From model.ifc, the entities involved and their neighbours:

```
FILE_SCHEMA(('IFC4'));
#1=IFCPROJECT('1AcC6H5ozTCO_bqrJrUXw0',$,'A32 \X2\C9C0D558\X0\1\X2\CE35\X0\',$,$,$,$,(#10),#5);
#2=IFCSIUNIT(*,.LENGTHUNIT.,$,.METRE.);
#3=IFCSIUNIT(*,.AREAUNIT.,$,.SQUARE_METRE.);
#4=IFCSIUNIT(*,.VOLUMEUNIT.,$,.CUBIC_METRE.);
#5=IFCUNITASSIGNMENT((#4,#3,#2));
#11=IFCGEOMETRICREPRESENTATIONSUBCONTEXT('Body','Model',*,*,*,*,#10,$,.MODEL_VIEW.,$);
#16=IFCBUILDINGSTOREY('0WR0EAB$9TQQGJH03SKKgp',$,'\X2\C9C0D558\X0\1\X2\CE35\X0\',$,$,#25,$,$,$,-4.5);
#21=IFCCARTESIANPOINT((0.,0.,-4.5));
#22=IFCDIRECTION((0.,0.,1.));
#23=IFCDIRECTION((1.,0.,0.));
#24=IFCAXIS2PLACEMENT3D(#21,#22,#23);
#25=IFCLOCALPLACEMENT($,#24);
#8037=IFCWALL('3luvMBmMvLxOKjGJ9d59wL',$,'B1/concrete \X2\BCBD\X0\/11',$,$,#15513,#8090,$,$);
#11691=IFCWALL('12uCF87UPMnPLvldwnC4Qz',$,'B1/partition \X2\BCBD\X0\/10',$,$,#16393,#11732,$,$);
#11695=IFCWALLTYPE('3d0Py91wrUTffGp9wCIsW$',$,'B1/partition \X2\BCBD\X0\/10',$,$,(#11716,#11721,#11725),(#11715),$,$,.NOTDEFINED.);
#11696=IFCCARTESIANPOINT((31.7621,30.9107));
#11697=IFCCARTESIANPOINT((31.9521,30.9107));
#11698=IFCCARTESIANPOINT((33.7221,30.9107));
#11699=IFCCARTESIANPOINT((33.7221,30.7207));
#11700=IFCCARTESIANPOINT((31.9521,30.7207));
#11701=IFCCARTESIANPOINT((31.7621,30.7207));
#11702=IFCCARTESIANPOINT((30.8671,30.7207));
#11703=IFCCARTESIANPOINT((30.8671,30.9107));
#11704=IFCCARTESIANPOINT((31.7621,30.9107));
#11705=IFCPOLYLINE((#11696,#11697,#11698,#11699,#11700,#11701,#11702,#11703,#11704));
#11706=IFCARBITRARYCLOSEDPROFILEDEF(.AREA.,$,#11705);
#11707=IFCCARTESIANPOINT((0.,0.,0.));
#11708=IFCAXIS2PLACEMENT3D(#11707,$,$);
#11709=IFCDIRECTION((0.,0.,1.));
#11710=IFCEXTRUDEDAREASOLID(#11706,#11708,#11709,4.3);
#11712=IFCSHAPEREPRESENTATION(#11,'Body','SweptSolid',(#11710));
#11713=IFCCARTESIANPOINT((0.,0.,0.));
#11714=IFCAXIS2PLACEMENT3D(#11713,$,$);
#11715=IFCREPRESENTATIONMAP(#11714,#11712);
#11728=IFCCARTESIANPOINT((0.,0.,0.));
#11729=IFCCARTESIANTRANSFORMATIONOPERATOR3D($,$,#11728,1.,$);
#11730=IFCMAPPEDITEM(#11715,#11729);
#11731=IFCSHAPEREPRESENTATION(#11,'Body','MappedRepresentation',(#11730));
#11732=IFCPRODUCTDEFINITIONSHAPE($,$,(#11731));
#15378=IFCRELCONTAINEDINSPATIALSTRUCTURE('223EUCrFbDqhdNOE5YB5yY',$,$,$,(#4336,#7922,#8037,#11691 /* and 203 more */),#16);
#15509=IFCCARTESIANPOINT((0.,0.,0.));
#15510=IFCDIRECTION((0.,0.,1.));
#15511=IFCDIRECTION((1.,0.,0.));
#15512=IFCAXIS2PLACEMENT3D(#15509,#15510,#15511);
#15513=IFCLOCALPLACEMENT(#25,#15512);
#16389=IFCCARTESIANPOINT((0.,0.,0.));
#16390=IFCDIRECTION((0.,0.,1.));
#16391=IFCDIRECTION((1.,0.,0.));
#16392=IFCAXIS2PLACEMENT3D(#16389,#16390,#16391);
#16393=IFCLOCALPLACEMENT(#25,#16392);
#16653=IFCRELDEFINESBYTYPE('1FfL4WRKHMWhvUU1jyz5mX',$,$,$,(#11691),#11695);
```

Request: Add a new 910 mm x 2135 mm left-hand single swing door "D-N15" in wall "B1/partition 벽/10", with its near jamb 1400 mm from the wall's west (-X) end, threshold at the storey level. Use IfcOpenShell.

```python
import numpy as np
import ifcopenshell
import ifcopenshell.api.feature
import ifcopenshell.api.geometry
import ifcopenshell.api.root
import ifcopenshell.api.spatial
import ifcopenshell.geom
import ifcopenshell.util.element
import ifcopenshell.util.placement
import ifcopenshell.util.representation
import ifcopenshell.util.shape
import ifcopenshell.util.unit

model = ifcopenshell.open("model.ifc")
unit_scale = ifcopenshell.util.unit.calculate_unit_scale(model)
settings = ifcopenshell.geom.settings()


def volume(element):
    """Net volume in cubic metres, openings subtracted."""
    shape = ifcopenshell.geom.create_shape(settings, element)
    return ifcopenshell.util.shape.get_volume(shape.geometry)


wall = model.by_guid("12uCF87UPMnPLvldwnC4Qz")
storey = ifcopenshell.util.element.get_container(wall, ifc_class="IfcBuildingStorey")
context = ifcopenshell.util.representation.get_context(model, "Model", "Body", "MODEL_VIEW")
before = volume(wall)

width, height, from_end, sill = 0.91, 2.135, 1.4, 0.0  # metres

# The wall runs along its own X axis, and the end named is its -X end.
wall_shape = ifcopenshell.geom.create_shape(settings, wall)
x, y, z = ifcopenshell.util.shape.get_vertices(wall_shape.geometry).T
start = x.min() + from_end
face, thickness = float(y.min()), float(y.max() - y.min())
wall_matrix = ifcopenshell.util.placement.get_local_placement(wall.ObjectPlacement)
level = ifcopenshell.util.placement.get_local_placement(storey.ObjectPlacement)[2, 3]


def in_wall(x, y):
    """Placement at x, y metres in the wall's axes, at sill height."""
    matrix = wall_matrix.copy()
    matrix[:, 3] = wall_matrix @ np.array([x / unit_scale, y / unit_scale, 0.0, 1.0])
    matrix[2, 3] = level + sill / unit_scale
    return matrix


# Opening: a box that overshoots both wall faces by 50 mm.
opening = ifcopenshell.api.root.create_entity(model, ifc_class="IfcOpeningElement", predefined_type="OPENING")
box = ifcopenshell.api.geometry.add_wall_representation(
    model, context=context, length=width, height=height, thickness=thickness + 0.1
)
ifcopenshell.api.geometry.assign_representation(model, product=opening, representation=box)
ifcopenshell.api.geometry.edit_object_placement(model, product=opening, matrix=in_wall(start, face - 0.05), is_si=False)
ifcopenshell.api.feature.add_feature(model, feature=opening, element=wall)

door = ifcopenshell.api.root.create_entity(model, ifc_class="IfcDoor", name="D-N15", predefined_type="DOOR")
door.OverallWidth, door.OverallHeight = width / unit_scale, height / unit_scale
door.OperationType = "SINGLE_SWING_LEFT"
body = ifcopenshell.api.geometry.add_door_representation(
    model,
    context=context,
    overall_width=door.OverallWidth,
    overall_height=door.OverallHeight,
    operation_type="SINGLE_SWING_LEFT",
    lining_properties={"LiningDepth": thickness / unit_scale, "ThresholdDepth": thickness / unit_scale},
)
ifcopenshell.api.geometry.assign_representation(model, product=door, representation=body)
ifcopenshell.api.spatial.assign_container(model, products=[door], relating_structure=storey)
ifcopenshell.api.feature.add_filling(model, opening=opening, element=door)

# The lining spans the wall, so the door starts at the wall face.
ifcopenshell.api.geometry.edit_object_placement(model, product=door, matrix=in_wall(start, face), is_si=False)

after = volume(wall)

print(f"wall volume {before:.3f} -> {after:.3f} m3")

model.write("model_rev.ifc")
```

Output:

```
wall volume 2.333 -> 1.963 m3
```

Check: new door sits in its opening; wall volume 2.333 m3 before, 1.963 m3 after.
